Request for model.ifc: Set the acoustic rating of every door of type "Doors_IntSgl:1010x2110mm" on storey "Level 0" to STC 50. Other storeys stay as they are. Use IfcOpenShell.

First a look at what the model holds.

```python
import ifcopenshell
import ifcopenshell.util.element

model = ifcopenshell.open("model.ifc")
print(model.schema)
storey = next(s for s in model.by_type("IfcBuildingStorey") if s.Name == "Level 0")
doors = [e for e in ifcopenshell.util.element.get_decomposition(storey) if e.is_a("IfcDoor")]
seen = {}
for e in doors:
    element_type = ifcopenshell.util.element.get_type(e)
    key = (element_type.Name if element_type != e and element_type else None, ifcopenshell.util.element.get_pset(e, "Pset_DoorCommon", "AcousticRating"))
    seen[key] = seen.get(key, 0) + 1
for (name, value), count in sorted(seen.items(), key=str):
    print(count, "x", name, "|", value)
```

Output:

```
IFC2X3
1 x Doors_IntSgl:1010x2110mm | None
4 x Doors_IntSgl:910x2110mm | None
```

```python
import ifcopenshell
import ifcopenshell.api.pset
import ifcopenshell.util.element

model = ifcopenshell.open("model.ifc")

storey = next(s for s in model.by_type("IfcBuildingStorey") if s.Name == "Level 0")
doors = [e for e in ifcopenshell.util.element.get_decomposition(storey) if e.is_a("IfcDoor")]

count = 0
for e in doors:
    element_type = ifcopenshell.util.element.get_type(e)
    if element_type in (None, e) or element_type.Name != "Doors_IntSgl:1010x2110mm":
        continue
    # add_pset returns the element's existing set when there is one.
    pset = ifcopenshell.api.pset.add_pset(model, product=e, name="Pset_DoorCommon")
    ifcopenshell.api.pset.edit_pset(model, pset=pset, properties={"AcousticRating": "STC 50"})
    count += 1

print(count, "doors updated")

model.write("model_edited.ifc")
```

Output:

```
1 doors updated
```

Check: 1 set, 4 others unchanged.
